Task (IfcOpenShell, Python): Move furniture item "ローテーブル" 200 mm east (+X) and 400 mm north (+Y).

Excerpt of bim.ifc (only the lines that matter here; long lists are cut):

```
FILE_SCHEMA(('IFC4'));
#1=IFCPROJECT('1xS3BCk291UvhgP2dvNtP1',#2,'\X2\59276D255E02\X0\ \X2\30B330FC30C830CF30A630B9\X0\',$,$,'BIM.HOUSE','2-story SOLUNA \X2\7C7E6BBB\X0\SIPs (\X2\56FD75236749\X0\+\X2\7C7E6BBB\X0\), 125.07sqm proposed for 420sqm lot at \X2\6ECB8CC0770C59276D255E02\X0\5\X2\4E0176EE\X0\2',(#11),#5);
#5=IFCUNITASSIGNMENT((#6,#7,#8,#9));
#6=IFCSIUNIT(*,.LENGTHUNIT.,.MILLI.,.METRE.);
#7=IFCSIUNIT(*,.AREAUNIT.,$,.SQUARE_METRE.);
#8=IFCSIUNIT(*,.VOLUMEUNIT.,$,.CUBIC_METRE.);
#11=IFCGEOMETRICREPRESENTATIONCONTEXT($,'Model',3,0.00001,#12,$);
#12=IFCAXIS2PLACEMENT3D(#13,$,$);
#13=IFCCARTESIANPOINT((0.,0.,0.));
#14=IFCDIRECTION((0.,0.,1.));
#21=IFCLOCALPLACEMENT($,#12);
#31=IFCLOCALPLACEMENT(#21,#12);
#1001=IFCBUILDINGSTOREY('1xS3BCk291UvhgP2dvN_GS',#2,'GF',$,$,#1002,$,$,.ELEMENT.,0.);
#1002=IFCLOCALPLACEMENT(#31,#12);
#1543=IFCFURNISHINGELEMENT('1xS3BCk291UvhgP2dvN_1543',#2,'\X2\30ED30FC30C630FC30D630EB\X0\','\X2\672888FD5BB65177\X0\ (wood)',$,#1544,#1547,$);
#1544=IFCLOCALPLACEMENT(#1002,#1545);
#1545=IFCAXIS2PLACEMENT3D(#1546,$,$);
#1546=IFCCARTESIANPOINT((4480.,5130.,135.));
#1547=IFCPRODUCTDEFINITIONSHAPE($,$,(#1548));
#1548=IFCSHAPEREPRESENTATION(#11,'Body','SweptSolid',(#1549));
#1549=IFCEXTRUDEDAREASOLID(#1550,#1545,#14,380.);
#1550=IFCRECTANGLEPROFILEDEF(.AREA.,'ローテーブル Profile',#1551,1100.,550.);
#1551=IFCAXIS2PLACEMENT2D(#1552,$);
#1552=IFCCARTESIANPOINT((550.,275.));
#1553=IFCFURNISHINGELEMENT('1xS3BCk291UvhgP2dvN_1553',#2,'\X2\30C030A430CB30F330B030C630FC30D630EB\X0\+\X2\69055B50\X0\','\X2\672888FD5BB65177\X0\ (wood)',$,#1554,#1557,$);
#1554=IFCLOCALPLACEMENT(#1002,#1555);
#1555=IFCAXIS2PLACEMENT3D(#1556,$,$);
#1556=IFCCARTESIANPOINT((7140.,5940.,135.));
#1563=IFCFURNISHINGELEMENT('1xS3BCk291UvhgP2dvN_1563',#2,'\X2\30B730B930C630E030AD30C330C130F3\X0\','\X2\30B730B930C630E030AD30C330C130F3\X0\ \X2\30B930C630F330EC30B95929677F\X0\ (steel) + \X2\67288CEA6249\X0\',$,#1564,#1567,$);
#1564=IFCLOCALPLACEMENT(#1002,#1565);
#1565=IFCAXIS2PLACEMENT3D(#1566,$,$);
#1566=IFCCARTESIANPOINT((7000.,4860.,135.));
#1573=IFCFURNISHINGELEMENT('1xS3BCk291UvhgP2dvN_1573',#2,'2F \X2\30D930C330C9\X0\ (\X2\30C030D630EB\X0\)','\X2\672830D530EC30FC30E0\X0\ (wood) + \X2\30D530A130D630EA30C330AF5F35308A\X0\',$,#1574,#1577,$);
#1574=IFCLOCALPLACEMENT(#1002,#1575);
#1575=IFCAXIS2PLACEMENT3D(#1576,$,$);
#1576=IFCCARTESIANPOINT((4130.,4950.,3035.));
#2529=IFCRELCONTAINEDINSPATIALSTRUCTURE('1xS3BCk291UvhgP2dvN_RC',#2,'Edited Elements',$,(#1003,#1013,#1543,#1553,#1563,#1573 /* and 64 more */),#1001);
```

```python
import ifcopenshell
import ifcopenshell.api.geometry
import ifcopenshell.util.placement
import ifcopenshell.util.unit

model = ifcopenshell.open("bim.ifc")
unit_scale = ifcopenshell.util.unit.calculate_unit_scale(model)

item = model.by_guid("1xS3BCk291UvhgP2dvN_1543")
matrix = ifcopenshell.util.placement.get_local_placement(item.ObjectPlacement)
matrix[0, 3] += 0.2 / unit_scale
matrix[1, 3] += 0.4 / unit_scale
ifcopenshell.api.geometry.edit_object_placement(model, product=item, matrix=matrix, is_si=False)

print(ifcopenshell.util.placement.get_local_placement(item.ObjectPlacement).round(3) + 0.0)

model.write("bim-out.ifc")
```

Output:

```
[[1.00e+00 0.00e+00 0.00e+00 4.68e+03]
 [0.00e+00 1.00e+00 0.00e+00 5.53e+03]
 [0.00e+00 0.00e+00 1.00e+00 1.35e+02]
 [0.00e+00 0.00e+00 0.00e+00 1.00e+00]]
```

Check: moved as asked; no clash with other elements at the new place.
